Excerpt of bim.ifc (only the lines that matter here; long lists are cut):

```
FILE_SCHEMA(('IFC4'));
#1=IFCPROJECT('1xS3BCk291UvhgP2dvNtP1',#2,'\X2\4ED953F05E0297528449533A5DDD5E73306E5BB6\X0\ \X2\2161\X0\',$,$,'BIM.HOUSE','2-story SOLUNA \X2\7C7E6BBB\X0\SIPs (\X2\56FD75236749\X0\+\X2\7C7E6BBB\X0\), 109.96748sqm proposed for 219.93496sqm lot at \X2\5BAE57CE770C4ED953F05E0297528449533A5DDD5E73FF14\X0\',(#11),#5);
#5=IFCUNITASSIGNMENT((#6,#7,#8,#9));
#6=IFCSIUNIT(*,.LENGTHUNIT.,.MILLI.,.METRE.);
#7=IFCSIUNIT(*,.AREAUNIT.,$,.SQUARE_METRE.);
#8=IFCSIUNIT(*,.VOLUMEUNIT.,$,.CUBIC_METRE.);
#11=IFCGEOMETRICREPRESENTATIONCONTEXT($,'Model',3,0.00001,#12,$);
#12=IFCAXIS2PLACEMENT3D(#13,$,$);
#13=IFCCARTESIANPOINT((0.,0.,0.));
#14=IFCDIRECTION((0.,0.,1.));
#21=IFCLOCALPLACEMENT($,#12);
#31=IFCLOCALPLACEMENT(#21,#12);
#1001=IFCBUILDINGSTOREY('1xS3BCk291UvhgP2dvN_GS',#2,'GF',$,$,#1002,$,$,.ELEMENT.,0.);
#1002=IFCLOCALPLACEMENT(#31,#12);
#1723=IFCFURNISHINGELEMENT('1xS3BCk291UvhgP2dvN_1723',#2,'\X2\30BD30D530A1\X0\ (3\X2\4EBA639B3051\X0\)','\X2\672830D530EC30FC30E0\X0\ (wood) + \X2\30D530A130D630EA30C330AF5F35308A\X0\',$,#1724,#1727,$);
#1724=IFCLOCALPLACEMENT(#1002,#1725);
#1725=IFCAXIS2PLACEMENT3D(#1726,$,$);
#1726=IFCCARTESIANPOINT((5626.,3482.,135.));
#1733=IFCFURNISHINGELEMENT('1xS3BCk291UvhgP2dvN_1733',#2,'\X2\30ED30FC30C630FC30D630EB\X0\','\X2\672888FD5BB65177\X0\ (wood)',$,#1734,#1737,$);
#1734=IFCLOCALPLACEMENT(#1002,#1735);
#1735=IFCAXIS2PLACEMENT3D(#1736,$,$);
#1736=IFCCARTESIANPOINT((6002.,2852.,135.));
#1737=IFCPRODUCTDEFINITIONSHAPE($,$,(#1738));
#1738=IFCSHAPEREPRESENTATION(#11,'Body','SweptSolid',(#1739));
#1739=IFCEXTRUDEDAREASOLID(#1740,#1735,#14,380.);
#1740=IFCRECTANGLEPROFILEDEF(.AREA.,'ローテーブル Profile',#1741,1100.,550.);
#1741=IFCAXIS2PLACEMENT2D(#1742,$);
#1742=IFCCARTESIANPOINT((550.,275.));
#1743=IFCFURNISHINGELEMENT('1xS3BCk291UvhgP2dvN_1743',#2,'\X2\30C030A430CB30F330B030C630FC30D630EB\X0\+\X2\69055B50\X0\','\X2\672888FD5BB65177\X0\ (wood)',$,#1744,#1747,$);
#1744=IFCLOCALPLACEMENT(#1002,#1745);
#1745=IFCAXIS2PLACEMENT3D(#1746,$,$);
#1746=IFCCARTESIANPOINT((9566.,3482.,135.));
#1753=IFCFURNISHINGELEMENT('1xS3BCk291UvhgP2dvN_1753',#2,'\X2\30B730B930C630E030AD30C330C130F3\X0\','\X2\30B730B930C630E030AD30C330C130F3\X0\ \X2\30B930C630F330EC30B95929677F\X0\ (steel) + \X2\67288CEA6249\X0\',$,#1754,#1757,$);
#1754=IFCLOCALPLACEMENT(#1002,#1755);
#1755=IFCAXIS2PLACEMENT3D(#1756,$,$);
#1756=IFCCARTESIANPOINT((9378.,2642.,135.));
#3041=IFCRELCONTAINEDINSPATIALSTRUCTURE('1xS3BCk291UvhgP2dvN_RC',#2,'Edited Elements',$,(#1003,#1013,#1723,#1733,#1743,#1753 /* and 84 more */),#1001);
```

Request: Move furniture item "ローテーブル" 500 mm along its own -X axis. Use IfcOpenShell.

```python
import ifcopenshell
import ifcopenshell.api.geometry
import ifcopenshell.util.placement
import ifcopenshell.util.unit

model = ifcopenshell.open("bim.ifc")
unit_scale = ifcopenshell.util.unit.calculate_unit_scale(model)

item = model.by_guid("1xS3BCk291UvhgP2dvN_1733")
matrix = ifcopenshell.util.placement.get_local_placement(item.ObjectPlacement)
matrix[:3, 3] -= matrix[:3, 0] * 0.5 / unit_scale
ifcopenshell.api.geometry.edit_object_placement(model, product=item, matrix=matrix, is_si=False)

print(ifcopenshell.util.placement.get_local_placement(item.ObjectPlacement).round(3) + 0.0)

model.write("bim_updated.ifc")
```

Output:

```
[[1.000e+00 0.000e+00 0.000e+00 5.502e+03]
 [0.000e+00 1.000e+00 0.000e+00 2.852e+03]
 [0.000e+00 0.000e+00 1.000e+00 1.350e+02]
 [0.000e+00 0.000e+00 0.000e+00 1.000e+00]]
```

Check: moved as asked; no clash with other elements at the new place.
